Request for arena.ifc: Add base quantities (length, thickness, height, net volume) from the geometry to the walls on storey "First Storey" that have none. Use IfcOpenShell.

First a look at what the model holds.

```python
import ifcopenshell
import ifcopenshell.util.element
import ifcopenshell.util.unit

model = ifcopenshell.open("arena.ifc")
print(model.schema)
for unit_type in ("LENGTHUNIT", "AREAUNIT", "VOLUMEUNIT"):
    print(unit_type, ifcopenshell.util.unit.calculate_unit_scale(model, unit_type))
storey = next(s for s in model.by_type("IfcBuildingStorey") if s.Name == "First Storey")
walls = [e for e in ifcopenshell.util.element.get_decomposition(storey) if e.is_a("IfcWall")]
for e in sorted(walls, key=lambda e: e.id()):
    print(e.id(), e.is_a(), e.Name, list(ifcopenshell.util.element.get_psets(e, qtos_only=True)), sep=" | ")
```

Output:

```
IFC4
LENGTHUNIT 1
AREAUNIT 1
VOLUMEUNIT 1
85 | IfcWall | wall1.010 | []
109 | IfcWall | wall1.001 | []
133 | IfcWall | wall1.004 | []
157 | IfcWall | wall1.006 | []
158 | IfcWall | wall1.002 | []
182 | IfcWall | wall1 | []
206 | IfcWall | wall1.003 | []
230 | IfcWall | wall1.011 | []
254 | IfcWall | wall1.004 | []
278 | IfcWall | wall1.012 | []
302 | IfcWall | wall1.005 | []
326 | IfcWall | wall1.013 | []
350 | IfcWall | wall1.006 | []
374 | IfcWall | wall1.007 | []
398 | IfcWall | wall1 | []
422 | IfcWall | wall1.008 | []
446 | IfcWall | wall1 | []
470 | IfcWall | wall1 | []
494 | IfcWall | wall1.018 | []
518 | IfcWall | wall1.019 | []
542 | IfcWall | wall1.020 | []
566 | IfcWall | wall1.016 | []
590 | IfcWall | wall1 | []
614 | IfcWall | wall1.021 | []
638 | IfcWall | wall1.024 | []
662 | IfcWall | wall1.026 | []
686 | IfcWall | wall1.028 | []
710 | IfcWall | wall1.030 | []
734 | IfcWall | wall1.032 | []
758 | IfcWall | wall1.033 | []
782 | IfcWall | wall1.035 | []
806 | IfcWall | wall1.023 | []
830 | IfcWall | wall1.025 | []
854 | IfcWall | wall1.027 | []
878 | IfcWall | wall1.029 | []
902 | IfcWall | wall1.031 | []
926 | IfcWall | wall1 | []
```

```python
import ifcopenshell
import ifcopenshell.api.pset
import ifcopenshell.geom
import ifcopenshell.util.element
import ifcopenshell.util.shape
import ifcopenshell.util.unit

model = ifcopenshell.open("arena.ifc")
unit_scale = ifcopenshell.util.unit.calculate_unit_scale(model)
volume_scale = ifcopenshell.util.unit.calculate_unit_scale(model, "VOLUMEUNIT")
settings = ifcopenshell.geom.settings()

storey = next(s for s in model.by_type("IfcBuildingStorey") if s.Name == "First Storey")
walls = [e for e in ifcopenshell.util.element.get_decomposition(storey) if e.is_a("IfcWall")]

for e in sorted(walls, key=lambda e: e.id()):
    if ifcopenshell.util.element.get_psets(e, qtos_only=True, should_inherit=False):
        continue
    # Geometry comes back in metres, in the element's own axes.
    shape = ifcopenshell.geom.create_shape(settings, e)
    values = {
        "Length": ifcopenshell.util.shape.get_x(shape.geometry) / unit_scale,
        "Width": ifcopenshell.util.shape.get_y(shape.geometry) / unit_scale,
        "Height": ifcopenshell.util.shape.get_z(shape.geometry) / unit_scale,
        "NetVolume": ifcopenshell.util.shape.get_volume(shape.geometry) / volume_scale,
    }
    qto = ifcopenshell.api.pset.add_qto(model, product=e, name="Qto_WallBaseQuantities")
    ifcopenshell.api.pset.edit_qto(model, qto=qto, properties=values)
    print(e.id(), {k: round(v, 3) for k, v in values.items()})

model.write("arena_rev.ifc")
```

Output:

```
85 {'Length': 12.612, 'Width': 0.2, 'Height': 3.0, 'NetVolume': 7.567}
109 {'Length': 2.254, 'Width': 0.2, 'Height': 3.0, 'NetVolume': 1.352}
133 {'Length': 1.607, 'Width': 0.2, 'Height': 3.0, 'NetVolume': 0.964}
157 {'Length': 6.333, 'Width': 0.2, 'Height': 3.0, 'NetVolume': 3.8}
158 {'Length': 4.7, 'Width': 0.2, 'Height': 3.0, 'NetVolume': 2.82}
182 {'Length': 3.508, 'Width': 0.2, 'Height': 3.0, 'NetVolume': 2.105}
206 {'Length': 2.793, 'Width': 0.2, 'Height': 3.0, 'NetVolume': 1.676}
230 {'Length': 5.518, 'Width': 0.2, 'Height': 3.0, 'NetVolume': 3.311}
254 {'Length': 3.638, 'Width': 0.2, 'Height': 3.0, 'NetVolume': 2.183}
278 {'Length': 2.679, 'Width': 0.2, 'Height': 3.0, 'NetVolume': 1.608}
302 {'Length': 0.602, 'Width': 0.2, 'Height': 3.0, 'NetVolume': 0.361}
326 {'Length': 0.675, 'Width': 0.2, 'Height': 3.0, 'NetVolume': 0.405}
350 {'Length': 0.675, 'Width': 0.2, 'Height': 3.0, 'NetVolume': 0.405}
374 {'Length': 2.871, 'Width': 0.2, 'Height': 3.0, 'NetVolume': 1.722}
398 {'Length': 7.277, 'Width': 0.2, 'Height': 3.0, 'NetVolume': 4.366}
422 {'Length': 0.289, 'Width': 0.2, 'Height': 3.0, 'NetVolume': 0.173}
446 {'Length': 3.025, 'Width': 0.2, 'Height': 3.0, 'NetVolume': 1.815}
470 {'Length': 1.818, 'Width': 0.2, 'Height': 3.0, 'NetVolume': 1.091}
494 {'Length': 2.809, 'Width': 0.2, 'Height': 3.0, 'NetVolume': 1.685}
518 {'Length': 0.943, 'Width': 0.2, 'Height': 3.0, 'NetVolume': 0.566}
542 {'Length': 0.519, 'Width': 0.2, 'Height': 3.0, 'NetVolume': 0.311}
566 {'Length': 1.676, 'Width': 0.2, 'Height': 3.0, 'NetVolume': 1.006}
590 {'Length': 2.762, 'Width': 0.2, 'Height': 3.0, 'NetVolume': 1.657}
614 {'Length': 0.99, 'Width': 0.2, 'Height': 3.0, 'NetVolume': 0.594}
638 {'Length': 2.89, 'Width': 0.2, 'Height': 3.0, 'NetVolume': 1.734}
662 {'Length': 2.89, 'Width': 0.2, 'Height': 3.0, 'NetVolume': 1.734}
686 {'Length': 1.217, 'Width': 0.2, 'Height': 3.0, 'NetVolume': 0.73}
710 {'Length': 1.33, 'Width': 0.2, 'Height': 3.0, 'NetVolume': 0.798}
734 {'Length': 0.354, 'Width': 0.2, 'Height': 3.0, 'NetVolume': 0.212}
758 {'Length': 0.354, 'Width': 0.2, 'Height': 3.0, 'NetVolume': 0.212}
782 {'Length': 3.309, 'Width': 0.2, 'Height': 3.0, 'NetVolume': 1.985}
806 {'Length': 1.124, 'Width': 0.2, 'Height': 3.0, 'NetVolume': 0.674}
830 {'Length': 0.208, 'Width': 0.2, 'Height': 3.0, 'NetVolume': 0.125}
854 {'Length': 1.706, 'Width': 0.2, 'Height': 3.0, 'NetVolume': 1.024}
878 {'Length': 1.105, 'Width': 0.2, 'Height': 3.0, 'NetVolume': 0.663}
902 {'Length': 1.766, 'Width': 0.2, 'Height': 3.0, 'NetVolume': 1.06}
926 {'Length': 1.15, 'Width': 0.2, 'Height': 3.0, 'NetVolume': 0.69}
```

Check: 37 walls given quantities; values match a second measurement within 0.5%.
